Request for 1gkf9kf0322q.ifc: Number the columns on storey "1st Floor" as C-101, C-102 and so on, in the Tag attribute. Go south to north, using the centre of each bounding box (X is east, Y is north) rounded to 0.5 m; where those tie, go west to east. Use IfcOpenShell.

First a look at what the model holds.

```python
import ifcopenshell
import ifcopenshell.util.element
import ifcopenshell.util.placement

model = ifcopenshell.open("1gkf9kf0322q.ifc")
print(model.schema)
storey = next(s for s in model.by_type("IfcBuildingStorey") if s.Name == "1st Floor")
columns = [e for e in ifcopenshell.util.element.get_decomposition(storey) if e.is_a("IfcColumn")]
for e in sorted(columns, key=lambda e: e.id()):
    origin = ifcopenshell.util.placement.get_local_placement(e.ObjectPlacement)[:3, 3]
    print(e.id(), e.Tag, e.Name, origin.round(2) + 0.0, sep=" | ")
```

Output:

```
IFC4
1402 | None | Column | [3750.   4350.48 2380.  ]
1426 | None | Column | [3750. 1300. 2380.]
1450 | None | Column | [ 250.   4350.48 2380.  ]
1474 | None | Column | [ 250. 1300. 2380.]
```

```python
import ifcopenshell
import ifcopenshell.geom
import ifcopenshell.util.element
import ifcopenshell.util.shape

model = ifcopenshell.open("1gkf9kf0322q.ifc")
settings = ifcopenshell.geom.settings()
settings.set("use-world-coords", True)


def centre(element):
    shape = ifcopenshell.geom.create_shape(settings, element)
    return ifcopenshell.util.shape.get_bbox_centroid(shape.geometry)


storey = next(s for s in model.by_type("IfcBuildingStorey") if s.Name == "1st Floor")
columns = [e for e in ifcopenshell.util.element.get_decomposition(storey) if e.is_a("IfcColumn")]

# Insertion points can sit at a corner or the storey origin, so sort by the geometry (in metres).
centres = {e: centre(e) for e in columns}
columns.sort(key=lambda e: (round(centres[e][1] / 0.5), centres[e][0]))

for i, e in enumerate(columns, start=1):
    number = f"C-1{i:02d}"
    e.Tag = number
    print(e.id(), number)

model.write("1gkf9kf0322q-out.ifc")
```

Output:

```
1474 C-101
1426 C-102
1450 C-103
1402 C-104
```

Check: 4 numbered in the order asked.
